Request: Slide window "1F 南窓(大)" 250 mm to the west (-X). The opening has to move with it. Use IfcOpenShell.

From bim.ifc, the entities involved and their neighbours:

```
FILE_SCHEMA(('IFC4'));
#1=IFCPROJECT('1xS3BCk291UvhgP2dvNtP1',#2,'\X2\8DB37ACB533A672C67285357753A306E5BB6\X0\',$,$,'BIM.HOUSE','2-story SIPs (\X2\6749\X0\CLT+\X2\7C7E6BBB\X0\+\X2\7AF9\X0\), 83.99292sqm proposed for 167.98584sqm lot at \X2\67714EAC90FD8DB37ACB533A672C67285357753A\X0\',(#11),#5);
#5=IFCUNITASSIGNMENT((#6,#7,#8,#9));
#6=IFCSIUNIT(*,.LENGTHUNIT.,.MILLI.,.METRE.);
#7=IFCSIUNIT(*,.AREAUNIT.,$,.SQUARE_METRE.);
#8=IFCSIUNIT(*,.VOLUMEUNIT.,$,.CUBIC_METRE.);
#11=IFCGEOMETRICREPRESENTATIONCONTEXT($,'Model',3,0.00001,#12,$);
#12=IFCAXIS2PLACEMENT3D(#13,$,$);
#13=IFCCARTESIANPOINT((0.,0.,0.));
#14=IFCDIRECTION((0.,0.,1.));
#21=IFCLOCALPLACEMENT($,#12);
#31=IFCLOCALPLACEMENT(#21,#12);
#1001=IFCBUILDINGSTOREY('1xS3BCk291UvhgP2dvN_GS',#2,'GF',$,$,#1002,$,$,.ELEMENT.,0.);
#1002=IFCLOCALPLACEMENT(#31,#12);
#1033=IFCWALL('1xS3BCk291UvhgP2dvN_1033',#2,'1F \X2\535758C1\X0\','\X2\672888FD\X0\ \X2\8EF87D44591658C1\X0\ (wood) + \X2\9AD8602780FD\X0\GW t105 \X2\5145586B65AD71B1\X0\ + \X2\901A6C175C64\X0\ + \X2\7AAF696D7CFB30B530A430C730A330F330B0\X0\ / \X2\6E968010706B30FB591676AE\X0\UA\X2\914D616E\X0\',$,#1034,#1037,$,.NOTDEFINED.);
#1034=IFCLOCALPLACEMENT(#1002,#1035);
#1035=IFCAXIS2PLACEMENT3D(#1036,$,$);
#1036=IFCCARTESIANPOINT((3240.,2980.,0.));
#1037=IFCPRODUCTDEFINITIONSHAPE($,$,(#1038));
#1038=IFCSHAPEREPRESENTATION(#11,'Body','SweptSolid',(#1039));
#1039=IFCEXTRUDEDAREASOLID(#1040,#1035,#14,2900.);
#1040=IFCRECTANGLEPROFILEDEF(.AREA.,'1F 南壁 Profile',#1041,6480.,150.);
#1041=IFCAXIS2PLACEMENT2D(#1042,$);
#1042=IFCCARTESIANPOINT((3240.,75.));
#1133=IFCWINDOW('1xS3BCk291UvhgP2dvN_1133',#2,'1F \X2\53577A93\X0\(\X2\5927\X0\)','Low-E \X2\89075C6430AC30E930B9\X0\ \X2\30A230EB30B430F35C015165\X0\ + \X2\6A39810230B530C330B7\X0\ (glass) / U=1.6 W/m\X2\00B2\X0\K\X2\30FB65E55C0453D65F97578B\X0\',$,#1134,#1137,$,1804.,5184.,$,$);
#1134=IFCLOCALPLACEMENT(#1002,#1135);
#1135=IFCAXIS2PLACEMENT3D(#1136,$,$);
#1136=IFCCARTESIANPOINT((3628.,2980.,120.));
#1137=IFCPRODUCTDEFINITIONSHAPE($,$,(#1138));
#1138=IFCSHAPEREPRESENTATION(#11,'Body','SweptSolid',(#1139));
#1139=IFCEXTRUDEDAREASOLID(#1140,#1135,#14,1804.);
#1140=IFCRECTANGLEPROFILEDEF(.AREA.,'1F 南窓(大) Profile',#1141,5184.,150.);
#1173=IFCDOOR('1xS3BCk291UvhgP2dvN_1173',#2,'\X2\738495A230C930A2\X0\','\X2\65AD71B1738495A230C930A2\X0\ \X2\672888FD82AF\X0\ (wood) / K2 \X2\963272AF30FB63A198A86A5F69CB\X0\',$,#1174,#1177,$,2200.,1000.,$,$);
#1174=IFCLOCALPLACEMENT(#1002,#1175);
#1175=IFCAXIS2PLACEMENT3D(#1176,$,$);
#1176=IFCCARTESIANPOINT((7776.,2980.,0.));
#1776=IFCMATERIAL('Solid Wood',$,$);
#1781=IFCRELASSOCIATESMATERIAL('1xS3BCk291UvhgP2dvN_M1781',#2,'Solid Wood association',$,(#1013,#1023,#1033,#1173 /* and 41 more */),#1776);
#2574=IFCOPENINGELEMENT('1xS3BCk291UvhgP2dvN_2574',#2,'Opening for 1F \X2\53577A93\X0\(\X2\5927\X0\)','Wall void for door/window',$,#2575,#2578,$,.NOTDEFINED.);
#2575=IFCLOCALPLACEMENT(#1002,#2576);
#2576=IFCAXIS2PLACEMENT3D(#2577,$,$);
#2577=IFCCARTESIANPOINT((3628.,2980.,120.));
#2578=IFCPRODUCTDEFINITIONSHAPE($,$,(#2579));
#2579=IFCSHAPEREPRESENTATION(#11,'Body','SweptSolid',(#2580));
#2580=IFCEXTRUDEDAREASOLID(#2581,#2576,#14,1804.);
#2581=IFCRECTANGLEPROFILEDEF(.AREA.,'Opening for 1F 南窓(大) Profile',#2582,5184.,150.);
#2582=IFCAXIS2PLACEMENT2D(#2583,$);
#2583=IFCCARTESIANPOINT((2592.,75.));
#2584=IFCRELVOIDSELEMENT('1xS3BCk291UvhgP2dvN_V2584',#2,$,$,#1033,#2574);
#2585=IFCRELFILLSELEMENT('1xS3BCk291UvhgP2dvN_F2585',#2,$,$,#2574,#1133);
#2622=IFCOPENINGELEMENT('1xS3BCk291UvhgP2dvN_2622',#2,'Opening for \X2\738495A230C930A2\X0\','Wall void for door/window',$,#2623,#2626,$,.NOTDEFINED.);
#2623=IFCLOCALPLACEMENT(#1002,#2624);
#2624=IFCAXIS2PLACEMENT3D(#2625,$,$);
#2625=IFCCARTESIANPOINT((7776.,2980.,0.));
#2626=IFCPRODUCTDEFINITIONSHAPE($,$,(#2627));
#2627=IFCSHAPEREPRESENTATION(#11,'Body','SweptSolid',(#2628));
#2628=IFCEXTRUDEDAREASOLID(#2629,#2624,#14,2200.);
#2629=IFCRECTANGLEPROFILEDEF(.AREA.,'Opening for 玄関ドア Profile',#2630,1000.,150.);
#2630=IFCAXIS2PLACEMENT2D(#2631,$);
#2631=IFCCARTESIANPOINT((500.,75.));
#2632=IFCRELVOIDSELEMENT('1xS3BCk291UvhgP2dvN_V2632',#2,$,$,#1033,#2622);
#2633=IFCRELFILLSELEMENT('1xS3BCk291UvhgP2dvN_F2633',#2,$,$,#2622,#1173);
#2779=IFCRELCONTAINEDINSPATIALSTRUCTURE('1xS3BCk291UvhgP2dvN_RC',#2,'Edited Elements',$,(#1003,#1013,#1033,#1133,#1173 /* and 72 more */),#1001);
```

```python
import ifcopenshell
import ifcopenshell.api.geometry
import ifcopenshell.util.placement

model = ifcopenshell.open("bim.ifc")

window = model.by_guid("1xS3BCk291UvhgP2dvN_1133")
opening = window.FillsVoids[0].RelatingOpeningElement
wall = opening.VoidsElements[0].RelatingBuildingElement

wall_matrix = ifcopenshell.util.placement.get_local_placement(wall.ObjectPlacement)
shift = wall_matrix[:3, 0] * -250.0
before = ifcopenshell.util.placement.get_local_placement(window.ObjectPlacement)[:3, 3].copy()

# The window is not placed relative to its opening, so move both.
for product in (opening, window):
    matrix = ifcopenshell.util.placement.get_local_placement(product.ObjectPlacement)
    matrix[:3, 3] += shift
    ifcopenshell.api.geometry.edit_object_placement(model, product=product, matrix=matrix, is_si=False)

after = ifcopenshell.util.placement.get_local_placement(window.ObjectPlacement)[:3, 3]
print("window moved by", (after - before).round(3) + 0.0)

model.write("bim-out.ifc")
```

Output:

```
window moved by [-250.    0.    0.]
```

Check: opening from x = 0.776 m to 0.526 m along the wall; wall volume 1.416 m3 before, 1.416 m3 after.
